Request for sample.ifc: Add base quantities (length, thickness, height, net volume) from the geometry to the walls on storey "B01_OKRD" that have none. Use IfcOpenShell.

First a look at what the model holds.

```python
import ifcopenshell
import ifcopenshell.util.element
import ifcopenshell.util.unit

model = ifcopenshell.open("sample.ifc")
print(model.schema)
for unit_type in ("LENGTHUNIT", "AREAUNIT", "VOLUMEUNIT"):
    print(unit_type, ifcopenshell.util.unit.calculate_unit_scale(model, unit_type))
storey = next(s for s in model.by_type("IfcBuildingStorey") if s.Name == "B01_OKRD")
walls = [e for e in ifcopenshell.util.element.get_decomposition(storey) if e.is_a("IfcWall")]
for e in sorted(walls, key=lambda e: e.id()):
    print(e.id(), e.is_a(), e.Name, list(ifcopenshell.util.element.get_psets(e, qtos_only=True)), sep=" | ")
```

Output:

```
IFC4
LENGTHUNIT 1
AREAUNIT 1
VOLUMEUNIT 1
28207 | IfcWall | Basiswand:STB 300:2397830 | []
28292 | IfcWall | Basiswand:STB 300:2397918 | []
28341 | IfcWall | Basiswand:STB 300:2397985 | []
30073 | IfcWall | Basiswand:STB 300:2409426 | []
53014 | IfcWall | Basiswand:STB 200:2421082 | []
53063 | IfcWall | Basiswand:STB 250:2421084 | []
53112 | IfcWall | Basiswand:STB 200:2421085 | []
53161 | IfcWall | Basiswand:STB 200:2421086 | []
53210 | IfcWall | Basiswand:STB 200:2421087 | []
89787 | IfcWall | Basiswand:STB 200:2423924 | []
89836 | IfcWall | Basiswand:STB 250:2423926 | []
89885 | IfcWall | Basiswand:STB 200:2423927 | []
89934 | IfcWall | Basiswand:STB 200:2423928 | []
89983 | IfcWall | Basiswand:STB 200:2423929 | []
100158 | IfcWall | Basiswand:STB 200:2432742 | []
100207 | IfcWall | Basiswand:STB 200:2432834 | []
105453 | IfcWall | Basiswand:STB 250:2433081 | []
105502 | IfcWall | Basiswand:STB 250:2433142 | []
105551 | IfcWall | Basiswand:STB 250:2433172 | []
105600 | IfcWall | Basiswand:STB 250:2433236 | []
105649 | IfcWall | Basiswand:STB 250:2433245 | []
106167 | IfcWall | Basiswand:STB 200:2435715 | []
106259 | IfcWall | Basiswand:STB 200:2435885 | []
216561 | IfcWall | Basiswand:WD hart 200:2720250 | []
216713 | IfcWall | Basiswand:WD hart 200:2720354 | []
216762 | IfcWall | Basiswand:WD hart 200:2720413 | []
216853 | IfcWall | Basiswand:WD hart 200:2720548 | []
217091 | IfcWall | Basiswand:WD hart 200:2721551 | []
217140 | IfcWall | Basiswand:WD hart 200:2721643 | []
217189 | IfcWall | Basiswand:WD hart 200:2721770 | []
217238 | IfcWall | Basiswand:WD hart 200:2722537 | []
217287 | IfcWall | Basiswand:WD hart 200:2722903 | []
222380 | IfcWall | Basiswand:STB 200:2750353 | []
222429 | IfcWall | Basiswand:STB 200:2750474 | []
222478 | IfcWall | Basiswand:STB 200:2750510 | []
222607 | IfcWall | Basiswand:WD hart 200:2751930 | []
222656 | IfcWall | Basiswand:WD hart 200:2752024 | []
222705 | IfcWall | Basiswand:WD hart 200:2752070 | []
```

```python
import ifcopenshell
import ifcopenshell.api.pset
import ifcopenshell.geom
import ifcopenshell.util.element
import ifcopenshell.util.shape
import ifcopenshell.util.unit

model = ifcopenshell.open("sample.ifc")
unit_scale = ifcopenshell.util.unit.calculate_unit_scale(model)
volume_scale = ifcopenshell.util.unit.calculate_unit_scale(model, "VOLUMEUNIT")
settings = ifcopenshell.geom.settings()

storey = next(s for s in model.by_type("IfcBuildingStorey") if s.Name == "B01_OKRD")
walls = [e for e in ifcopenshell.util.element.get_decomposition(storey) if e.is_a("IfcWall")]

for e in sorted(walls, key=lambda e: e.id()):
    if ifcopenshell.util.element.get_psets(e, qtos_only=True, should_inherit=False):
        continue
    # Geometry comes back in metres, in the element's own axes.
    shape = ifcopenshell.geom.create_shape(settings, e)
    values = {
        "Length": ifcopenshell.util.shape.get_x(shape.geometry) / unit_scale,
        "Width": ifcopenshell.util.shape.get_y(shape.geometry) / unit_scale,
        "Height": ifcopenshell.util.shape.get_z(shape.geometry) / unit_scale,
        "NetVolume": ifcopenshell.util.shape.get_volume(shape.geometry) / volume_scale,
    }
    qto = ifcopenshell.api.pset.add_qto(model, product=e, name="Qto_WallBaseQuantities")
    ifcopenshell.api.pset.edit_qto(model, qto=qto, properties=values)
    print(e.id(), {k: round(v, 3) for k, v in values.items()})

model.write("sample_edited.ifc")
```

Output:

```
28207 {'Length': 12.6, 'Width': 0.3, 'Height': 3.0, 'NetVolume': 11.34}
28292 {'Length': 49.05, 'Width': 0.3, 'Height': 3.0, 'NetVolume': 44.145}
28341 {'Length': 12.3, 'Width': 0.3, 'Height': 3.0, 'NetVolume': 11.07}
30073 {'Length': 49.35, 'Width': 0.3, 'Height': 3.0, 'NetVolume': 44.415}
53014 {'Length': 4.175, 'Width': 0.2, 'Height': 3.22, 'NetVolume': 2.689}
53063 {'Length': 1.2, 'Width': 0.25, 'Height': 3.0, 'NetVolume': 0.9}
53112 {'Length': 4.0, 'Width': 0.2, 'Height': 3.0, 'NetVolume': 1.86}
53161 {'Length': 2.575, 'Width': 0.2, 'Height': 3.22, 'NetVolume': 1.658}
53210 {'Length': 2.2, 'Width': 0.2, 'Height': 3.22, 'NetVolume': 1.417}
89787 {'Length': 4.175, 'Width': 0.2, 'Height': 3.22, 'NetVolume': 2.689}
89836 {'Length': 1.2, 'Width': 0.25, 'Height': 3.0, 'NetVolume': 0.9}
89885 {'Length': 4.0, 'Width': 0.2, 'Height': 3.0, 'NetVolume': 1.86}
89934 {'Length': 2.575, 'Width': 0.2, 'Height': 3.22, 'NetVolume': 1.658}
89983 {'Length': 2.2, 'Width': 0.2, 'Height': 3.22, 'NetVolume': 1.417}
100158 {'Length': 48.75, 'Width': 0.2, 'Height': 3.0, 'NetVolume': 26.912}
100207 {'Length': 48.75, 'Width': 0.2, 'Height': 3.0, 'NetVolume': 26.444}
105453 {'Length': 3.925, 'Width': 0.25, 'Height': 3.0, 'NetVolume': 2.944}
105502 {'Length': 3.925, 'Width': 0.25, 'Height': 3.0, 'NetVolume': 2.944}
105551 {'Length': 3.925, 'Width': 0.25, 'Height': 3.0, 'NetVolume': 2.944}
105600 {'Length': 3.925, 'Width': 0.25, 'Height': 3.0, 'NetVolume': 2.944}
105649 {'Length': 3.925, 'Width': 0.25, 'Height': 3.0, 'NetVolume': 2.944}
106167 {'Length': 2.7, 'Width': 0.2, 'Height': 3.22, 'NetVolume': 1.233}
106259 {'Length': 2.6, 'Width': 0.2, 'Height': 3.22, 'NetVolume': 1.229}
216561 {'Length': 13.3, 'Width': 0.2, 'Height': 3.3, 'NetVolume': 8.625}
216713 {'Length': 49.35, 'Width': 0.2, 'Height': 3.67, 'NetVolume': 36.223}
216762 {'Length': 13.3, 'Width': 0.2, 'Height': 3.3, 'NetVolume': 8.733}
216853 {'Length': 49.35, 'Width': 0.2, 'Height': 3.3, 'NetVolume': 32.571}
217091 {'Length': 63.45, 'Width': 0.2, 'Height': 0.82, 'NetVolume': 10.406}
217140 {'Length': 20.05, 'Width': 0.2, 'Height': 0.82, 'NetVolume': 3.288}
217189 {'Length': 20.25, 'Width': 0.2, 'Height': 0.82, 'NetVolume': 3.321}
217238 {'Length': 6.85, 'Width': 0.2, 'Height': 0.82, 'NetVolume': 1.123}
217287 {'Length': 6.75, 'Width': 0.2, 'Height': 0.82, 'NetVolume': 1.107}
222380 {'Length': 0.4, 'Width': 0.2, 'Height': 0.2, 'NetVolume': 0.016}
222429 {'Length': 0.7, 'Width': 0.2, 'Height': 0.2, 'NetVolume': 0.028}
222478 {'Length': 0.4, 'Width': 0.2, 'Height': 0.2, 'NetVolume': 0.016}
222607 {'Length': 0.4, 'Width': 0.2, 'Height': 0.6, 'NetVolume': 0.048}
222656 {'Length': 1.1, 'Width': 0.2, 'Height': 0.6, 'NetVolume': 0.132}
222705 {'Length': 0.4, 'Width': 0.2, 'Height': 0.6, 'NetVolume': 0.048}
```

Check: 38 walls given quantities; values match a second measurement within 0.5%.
